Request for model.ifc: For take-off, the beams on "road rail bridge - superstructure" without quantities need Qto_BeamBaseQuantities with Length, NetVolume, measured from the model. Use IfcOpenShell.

First a look at what the model holds.

```python
import ifcopenshell
import ifcopenshell.util.element
import ifcopenshell.util.unit

model = ifcopenshell.open("model.ifc")
print(model.schema)
for unit_type in ("LENGTHUNIT", "AREAUNIT", "VOLUMEUNIT"):
    print(unit_type, ifcopenshell.util.unit.calculate_unit_scale(model, unit_type))
storey = next(s for s in model.by_type("IfcBuildingStorey") if s.Name == "road rail bridge - superstructure")
beams = [e for e in ifcopenshell.util.element.get_decomposition(storey) if e.is_a("IfcBeam")]
for e in sorted(beams, key=lambda e: e.id()):
    print(e.id(), e.is_a(), e.Name, list(ifcopenshell.util.element.get_psets(e, qtos_only=True)), sep=" | ")
```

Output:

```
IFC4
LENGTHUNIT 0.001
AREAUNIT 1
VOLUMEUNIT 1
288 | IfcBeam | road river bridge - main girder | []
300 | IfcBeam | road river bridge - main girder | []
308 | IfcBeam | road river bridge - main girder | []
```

```python
import ifcopenshell
import ifcopenshell.api.pset
import ifcopenshell.geom
import ifcopenshell.util.element
import ifcopenshell.util.shape
import ifcopenshell.util.unit

model = ifcopenshell.open("model.ifc")
unit_scale = ifcopenshell.util.unit.calculate_unit_scale(model)
volume_scale = ifcopenshell.util.unit.calculate_unit_scale(model, "VOLUMEUNIT")
settings = ifcopenshell.geom.settings()

storey = next(s for s in model.by_type("IfcBuildingStorey") if s.Name == "road rail bridge - superstructure")
beams = [e for e in ifcopenshell.util.element.get_decomposition(storey) if e.is_a("IfcBeam")]

for e in sorted(beams, key=lambda e: e.id()):
    if ifcopenshell.util.element.get_psets(e, qtos_only=True, should_inherit=False):
        continue
    # Geometry comes back in metres, in the element's own axes.
    shape = ifcopenshell.geom.create_shape(settings, e)
    values = {
        "Length": ifcopenshell.util.shape.get_max_xyz(shape.geometry) / unit_scale,
        "NetVolume": ifcopenshell.util.shape.get_volume(shape.geometry) / volume_scale,
    }
    qto = ifcopenshell.api.pset.add_qto(model, product=e, name="Qto_BeamBaseQuantities")
    ifcopenshell.api.pset.edit_qto(model, qto=qto, properties=values)
    print(e.id(), {k: round(v, 3) for k, v in values.items()})

model.write("model_edited.ifc")
```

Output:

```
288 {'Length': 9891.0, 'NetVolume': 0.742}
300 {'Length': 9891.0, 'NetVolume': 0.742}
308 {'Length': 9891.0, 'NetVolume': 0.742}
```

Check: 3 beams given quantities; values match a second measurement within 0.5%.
